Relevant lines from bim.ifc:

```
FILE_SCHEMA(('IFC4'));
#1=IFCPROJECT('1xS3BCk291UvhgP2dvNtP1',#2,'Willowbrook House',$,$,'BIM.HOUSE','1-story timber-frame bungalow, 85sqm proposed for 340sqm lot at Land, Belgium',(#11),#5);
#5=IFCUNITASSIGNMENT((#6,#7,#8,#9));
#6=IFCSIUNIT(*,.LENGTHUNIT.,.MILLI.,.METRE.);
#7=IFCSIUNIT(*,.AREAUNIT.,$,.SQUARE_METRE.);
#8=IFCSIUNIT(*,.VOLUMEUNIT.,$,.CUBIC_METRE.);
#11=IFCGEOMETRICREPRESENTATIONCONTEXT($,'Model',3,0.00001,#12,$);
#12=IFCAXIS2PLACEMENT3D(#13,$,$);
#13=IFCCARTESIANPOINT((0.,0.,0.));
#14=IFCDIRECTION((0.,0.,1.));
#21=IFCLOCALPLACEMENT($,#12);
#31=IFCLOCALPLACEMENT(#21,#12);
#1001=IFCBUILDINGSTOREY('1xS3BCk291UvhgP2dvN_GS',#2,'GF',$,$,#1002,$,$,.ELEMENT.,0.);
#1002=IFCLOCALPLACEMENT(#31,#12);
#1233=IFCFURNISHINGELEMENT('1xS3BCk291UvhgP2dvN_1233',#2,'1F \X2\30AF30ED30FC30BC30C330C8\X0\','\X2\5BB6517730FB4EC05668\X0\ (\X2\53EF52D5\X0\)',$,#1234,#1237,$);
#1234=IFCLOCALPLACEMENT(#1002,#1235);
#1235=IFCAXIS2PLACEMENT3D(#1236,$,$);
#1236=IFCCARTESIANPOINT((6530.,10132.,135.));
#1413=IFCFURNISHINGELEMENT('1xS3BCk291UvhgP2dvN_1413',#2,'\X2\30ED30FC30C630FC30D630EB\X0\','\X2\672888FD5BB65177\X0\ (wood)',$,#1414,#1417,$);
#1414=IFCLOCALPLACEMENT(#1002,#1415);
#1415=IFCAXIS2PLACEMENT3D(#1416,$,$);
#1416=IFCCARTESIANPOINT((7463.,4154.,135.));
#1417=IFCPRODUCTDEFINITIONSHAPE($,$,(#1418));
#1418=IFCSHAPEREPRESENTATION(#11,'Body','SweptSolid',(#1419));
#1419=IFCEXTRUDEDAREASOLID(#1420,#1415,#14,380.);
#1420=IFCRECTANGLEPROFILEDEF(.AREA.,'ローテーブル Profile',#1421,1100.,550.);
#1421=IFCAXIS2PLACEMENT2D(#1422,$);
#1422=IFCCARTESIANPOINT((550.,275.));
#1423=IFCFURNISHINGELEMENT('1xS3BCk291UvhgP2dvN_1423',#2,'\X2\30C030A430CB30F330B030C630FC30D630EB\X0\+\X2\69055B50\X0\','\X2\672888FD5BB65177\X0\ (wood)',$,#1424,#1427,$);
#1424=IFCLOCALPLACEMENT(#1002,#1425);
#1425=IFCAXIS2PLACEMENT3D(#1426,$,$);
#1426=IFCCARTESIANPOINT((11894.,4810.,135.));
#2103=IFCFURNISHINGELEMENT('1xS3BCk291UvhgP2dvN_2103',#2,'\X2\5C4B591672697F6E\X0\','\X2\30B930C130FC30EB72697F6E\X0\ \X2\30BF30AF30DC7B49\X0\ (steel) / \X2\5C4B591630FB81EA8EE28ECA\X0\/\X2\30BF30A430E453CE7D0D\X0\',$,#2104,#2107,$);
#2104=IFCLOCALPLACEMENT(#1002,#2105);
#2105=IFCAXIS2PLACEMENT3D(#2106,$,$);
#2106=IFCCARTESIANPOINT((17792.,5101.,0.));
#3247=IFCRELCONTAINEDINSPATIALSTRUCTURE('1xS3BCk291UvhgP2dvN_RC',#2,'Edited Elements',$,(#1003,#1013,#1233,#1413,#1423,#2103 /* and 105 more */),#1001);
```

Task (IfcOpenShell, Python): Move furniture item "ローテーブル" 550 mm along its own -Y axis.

```python
import ifcopenshell
import ifcopenshell.api.geometry
import ifcopenshell.util.placement
import ifcopenshell.util.unit

model = ifcopenshell.open("bim.ifc")
unit_scale = ifcopenshell.util.unit.calculate_unit_scale(model)

item = model.by_guid("1xS3BCk291UvhgP2dvN_1413")
matrix = ifcopenshell.util.placement.get_local_placement(item.ObjectPlacement)
matrix[:3, 3] -= matrix[:3, 1] * 0.55 / unit_scale
ifcopenshell.api.geometry.edit_object_placement(model, product=item, matrix=matrix, is_si=False)

print(ifcopenshell.util.placement.get_local_placement(item.ObjectPlacement).round(3) + 0.0)

model.write("bim_v2.ifc")
```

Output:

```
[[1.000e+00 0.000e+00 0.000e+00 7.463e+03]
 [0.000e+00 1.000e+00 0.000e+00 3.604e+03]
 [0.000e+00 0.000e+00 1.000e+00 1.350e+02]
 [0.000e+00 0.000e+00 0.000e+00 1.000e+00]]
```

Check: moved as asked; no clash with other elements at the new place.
